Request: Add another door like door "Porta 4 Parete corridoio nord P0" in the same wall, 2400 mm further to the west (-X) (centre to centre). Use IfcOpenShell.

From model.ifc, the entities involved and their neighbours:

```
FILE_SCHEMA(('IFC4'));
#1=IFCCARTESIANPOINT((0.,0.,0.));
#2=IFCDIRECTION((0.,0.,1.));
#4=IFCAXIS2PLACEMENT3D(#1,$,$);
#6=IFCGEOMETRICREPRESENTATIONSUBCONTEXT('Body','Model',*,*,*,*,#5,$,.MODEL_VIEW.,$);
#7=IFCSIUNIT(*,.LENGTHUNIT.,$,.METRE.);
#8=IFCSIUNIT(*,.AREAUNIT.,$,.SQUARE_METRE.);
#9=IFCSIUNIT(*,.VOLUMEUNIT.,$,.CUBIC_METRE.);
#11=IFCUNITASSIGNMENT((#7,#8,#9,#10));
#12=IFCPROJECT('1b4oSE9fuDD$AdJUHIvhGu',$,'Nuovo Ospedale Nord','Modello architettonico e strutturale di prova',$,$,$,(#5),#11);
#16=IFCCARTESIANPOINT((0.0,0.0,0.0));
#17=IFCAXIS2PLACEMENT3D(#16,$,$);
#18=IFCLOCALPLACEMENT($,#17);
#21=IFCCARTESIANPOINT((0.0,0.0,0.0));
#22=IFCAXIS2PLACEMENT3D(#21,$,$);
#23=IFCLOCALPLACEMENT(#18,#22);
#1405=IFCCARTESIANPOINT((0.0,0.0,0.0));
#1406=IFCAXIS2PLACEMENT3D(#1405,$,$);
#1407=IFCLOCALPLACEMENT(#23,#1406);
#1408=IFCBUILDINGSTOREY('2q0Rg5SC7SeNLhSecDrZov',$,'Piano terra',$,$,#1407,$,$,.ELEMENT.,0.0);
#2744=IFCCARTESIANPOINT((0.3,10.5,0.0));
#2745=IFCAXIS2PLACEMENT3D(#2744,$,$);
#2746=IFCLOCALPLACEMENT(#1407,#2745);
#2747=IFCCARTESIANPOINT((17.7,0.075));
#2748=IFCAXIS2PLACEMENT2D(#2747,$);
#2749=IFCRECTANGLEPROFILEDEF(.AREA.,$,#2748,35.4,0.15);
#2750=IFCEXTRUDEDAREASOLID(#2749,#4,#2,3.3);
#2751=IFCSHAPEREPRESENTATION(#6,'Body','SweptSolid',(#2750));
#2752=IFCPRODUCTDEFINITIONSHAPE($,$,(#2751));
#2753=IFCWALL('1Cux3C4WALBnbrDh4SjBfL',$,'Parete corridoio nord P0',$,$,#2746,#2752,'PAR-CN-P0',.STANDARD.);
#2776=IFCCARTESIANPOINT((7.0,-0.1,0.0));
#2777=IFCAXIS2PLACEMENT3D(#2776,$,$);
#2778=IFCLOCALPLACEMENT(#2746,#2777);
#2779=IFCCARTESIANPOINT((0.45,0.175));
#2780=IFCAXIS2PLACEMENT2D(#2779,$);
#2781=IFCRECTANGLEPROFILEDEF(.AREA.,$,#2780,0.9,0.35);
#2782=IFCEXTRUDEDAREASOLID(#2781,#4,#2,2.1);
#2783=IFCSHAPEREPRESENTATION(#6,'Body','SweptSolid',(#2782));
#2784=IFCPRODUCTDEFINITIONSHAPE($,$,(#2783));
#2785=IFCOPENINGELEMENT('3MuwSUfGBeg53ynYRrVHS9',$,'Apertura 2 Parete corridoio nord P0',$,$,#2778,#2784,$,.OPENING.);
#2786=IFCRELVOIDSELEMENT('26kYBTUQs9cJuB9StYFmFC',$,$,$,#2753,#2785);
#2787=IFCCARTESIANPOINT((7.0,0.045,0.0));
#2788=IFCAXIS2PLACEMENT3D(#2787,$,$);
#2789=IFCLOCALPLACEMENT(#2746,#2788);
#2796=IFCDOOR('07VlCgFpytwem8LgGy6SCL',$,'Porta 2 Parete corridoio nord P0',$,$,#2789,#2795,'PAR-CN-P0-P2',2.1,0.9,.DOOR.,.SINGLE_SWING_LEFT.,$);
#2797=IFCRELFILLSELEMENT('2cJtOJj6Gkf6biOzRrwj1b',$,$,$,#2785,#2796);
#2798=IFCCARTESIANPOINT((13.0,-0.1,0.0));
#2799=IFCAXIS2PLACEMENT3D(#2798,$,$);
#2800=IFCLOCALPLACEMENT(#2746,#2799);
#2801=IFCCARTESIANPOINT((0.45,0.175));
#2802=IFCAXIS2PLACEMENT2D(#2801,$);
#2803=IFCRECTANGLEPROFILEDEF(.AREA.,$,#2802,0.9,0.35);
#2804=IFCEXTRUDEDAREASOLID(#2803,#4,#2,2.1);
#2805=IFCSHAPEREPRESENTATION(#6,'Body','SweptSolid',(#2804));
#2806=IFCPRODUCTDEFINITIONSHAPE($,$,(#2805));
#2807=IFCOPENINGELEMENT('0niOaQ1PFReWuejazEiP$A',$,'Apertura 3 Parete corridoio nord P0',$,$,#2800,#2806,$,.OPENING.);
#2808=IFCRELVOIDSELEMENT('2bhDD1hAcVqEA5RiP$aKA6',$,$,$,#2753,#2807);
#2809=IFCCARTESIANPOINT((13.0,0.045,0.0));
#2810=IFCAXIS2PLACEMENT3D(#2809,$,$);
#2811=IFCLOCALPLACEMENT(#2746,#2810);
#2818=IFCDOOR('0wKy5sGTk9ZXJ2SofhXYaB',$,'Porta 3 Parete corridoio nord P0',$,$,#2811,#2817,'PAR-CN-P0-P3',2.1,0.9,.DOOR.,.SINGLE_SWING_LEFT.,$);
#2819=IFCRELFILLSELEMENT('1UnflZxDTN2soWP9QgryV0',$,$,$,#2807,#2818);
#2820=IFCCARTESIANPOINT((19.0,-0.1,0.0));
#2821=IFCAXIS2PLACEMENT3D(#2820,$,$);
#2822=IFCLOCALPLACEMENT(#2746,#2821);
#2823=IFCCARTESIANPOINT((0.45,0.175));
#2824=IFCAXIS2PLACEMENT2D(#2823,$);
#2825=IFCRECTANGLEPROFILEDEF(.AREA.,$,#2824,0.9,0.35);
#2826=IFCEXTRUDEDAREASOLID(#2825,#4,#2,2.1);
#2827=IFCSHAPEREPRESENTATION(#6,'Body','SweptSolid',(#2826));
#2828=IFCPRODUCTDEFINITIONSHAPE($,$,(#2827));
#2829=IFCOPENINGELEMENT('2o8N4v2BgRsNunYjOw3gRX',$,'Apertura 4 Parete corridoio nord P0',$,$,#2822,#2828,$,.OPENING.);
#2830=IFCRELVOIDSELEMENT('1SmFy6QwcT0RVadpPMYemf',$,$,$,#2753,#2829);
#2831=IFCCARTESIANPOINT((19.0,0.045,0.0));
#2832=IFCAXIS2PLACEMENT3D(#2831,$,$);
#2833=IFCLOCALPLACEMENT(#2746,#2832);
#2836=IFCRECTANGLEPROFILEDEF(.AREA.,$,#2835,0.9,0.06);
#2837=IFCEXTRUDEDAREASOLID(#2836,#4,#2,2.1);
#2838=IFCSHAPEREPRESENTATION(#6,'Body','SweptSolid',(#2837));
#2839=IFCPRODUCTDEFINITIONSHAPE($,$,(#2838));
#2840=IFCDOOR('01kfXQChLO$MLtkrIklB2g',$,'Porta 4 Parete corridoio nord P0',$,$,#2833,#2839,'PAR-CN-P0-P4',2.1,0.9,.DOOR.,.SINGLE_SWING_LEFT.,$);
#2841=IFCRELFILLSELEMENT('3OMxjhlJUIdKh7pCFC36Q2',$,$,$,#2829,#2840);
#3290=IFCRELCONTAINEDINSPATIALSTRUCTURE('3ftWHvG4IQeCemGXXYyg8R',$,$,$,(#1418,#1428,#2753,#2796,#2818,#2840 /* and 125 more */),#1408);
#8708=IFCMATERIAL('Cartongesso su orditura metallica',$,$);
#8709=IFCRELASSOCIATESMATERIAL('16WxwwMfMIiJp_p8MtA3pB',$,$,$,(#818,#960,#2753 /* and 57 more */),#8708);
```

```python
import ifcopenshell
import ifcopenshell.api.feature
import ifcopenshell.api.geometry
import ifcopenshell.api.root
import ifcopenshell.geom
import ifcopenshell.util.element
import ifcopenshell.util.placement
import ifcopenshell.util.shape
import ifcopenshell.util.unit

model = ifcopenshell.open("model.ifc")
unit_scale = ifcopenshell.util.unit.calculate_unit_scale(model)
settings = ifcopenshell.geom.settings()


def volume(element):
    """Net volume in cubic metres, openings subtracted."""
    shape = ifcopenshell.geom.create_shape(settings, element)
    return ifcopenshell.util.shape.get_volume(shape.geometry)


door = model.by_guid("01kfXQChLO$MLtkrIklB2g")
opening = door.FillsVoids[0].RelatingOpeningElement
wall = opening.VoidsElements[0].RelatingBuildingElement
before = volume(wall)
shift = ifcopenshell.util.placement.get_local_placement(wall.ObjectPlacement)[:3, 0] * -2.4 / unit_scale

# copy_class copies the void relationship, type, container and properties, but no geometry.
new_opening = ifcopenshell.api.root.copy_class(model, product=opening)
new_opening.Representation = ifcopenshell.util.element.copy_deep(
    model, opening.Representation, exclude=["IfcGeometricRepresentationContext", "IfcRepresentationMap"]
)
new_door = ifcopenshell.api.root.copy_class(model, product=door)
new_door.Representation = ifcopenshell.util.element.copy_deep(
    model, door.Representation, exclude=["IfcGeometricRepresentationContext", "IfcRepresentationMap"]
)
new_door.Tag = None
ifcopenshell.api.feature.add_filling(model, opening=new_opening, element=new_door)

for old, new in ((opening, new_opening), (door, new_door)):
    matrix = ifcopenshell.util.placement.get_local_placement(old.ObjectPlacement)
    matrix[:3, 3] += shift
    ifcopenshell.api.geometry.edit_object_placement(model, product=new, matrix=matrix, is_si=False)

after = volume(wall)

print(f"wall volume {before:.3f} -> {after:.3f} m3")

model.write("model_v2.ifc")
```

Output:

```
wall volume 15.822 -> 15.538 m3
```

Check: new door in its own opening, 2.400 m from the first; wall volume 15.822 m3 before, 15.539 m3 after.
